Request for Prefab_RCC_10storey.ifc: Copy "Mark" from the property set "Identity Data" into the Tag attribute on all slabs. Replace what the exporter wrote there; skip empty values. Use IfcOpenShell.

First a look at what the model holds.

```python
import ifcopenshell
import ifcopenshell.util.element

model = ifcopenshell.open("Prefab_RCC_10storey.ifc")
print(model.schema)
slabs = model.by_type("IfcSlab")
print(len(slabs), "slabs")
for e in slabs[:8]:
    source = ifcopenshell.util.element.get_pset(e, "Identity Data", "Mark")
    target = e.Tag
    print(e.id(), repr(source), repr(target), sep=" | ")
```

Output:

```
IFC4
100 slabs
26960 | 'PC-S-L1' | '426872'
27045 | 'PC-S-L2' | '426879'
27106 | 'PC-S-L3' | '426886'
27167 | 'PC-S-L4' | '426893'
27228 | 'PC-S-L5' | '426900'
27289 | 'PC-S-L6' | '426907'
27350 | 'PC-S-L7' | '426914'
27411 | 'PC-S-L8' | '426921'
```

```python
import ifcopenshell
import ifcopenshell.util.element

model = ifcopenshell.open("Prefab_RCC_10storey.ifc")

count = 0
for e in model.by_type("IfcSlab"):
    value = ifcopenshell.util.element.get_pset(e, "Identity Data", "Mark")
    current = e.Tag
    if not value or not value.strip() or current == value:
        continue
    e.Tag = value
    count += 1

print(count, "slabs updated")

model.write("Prefab_RCC_10storey-out.ifc")
```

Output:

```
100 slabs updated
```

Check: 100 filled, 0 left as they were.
